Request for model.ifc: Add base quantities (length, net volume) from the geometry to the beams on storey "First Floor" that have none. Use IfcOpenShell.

First a look at what the model holds.

```python
import ifcopenshell
import ifcopenshell.util.element
import ifcopenshell.util.unit

model = ifcopenshell.open("model.ifc")
print(model.schema)
for unit_type in ("LENGTHUNIT", "AREAUNIT", "VOLUMEUNIT"):
    print(unit_type, ifcopenshell.util.unit.calculate_unit_scale(model, unit_type))
storey = next(s for s in model.by_type("IfcBuildingStorey") if s.Name == "First Floor")
beams = [e for e in ifcopenshell.util.element.get_decomposition(storey) if e.is_a("IfcBeam")]
for e in sorted(beams, key=lambda e: e.id()):
    print(e.id(), e.is_a(), e.Name, list(ifcopenshell.util.element.get_psets(e, qtos_only=True)), sep=" | ")
```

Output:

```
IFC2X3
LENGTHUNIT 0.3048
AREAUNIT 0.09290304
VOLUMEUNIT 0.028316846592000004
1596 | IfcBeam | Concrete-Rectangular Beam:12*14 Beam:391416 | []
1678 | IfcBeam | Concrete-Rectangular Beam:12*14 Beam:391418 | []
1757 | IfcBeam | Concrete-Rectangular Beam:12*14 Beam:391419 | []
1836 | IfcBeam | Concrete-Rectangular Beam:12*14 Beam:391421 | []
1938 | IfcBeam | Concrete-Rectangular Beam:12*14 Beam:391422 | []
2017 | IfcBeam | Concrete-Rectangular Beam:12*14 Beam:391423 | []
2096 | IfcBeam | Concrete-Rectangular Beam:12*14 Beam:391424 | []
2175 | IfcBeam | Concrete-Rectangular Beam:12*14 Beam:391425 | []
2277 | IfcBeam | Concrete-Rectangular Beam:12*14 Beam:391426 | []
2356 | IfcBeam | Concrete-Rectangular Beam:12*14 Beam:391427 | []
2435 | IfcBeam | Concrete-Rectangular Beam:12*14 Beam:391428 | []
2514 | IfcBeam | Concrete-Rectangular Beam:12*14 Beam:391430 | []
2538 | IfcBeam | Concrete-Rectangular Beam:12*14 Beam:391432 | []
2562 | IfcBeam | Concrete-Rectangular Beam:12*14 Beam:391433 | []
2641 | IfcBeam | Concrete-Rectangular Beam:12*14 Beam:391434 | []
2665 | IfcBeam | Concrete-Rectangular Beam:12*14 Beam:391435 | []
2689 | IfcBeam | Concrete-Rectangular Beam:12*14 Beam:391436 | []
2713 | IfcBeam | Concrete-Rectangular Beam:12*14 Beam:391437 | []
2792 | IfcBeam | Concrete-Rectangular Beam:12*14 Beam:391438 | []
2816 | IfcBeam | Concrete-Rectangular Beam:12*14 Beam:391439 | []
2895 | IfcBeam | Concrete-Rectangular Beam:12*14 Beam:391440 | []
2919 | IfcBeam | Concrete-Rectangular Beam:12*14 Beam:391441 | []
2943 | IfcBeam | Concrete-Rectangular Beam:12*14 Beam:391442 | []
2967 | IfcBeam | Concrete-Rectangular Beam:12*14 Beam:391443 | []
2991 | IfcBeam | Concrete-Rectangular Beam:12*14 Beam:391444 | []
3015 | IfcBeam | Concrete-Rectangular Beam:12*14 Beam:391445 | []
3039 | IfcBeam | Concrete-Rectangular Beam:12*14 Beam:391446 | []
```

```python
import ifcopenshell
import ifcopenshell.api.pset
import ifcopenshell.geom
import ifcopenshell.util.element
import ifcopenshell.util.shape
import ifcopenshell.util.unit

model = ifcopenshell.open("model.ifc")
unit_scale = ifcopenshell.util.unit.calculate_unit_scale(model)
volume_scale = ifcopenshell.util.unit.calculate_unit_scale(model, "VOLUMEUNIT")
settings = ifcopenshell.geom.settings()

storey = next(s for s in model.by_type("IfcBuildingStorey") if s.Name == "First Floor")
beams = [e for e in ifcopenshell.util.element.get_decomposition(storey) if e.is_a("IfcBeam")]

for e in sorted(beams, key=lambda e: e.id()):
    if ifcopenshell.util.element.get_psets(e, qtos_only=True, should_inherit=False):
        continue
    # Geometry comes back in metres, in the element's own axes.
    shape = ifcopenshell.geom.create_shape(settings, e)
    values = {
        "Length": ifcopenshell.util.shape.get_max_xyz(shape.geometry) / unit_scale,
        "NetVolume": ifcopenshell.util.shape.get_volume(shape.geometry) / volume_scale,
    }
    qto = ifcopenshell.api.pset.add_qto(model, product=e, name="BaseQuantities")
    ifcopenshell.api.pset.edit_qto(model, qto=qto, properties=values)
    print(e.id(), {k: round(v, 3) for k, v in values.items()})

model.write("model_updated.ifc")
```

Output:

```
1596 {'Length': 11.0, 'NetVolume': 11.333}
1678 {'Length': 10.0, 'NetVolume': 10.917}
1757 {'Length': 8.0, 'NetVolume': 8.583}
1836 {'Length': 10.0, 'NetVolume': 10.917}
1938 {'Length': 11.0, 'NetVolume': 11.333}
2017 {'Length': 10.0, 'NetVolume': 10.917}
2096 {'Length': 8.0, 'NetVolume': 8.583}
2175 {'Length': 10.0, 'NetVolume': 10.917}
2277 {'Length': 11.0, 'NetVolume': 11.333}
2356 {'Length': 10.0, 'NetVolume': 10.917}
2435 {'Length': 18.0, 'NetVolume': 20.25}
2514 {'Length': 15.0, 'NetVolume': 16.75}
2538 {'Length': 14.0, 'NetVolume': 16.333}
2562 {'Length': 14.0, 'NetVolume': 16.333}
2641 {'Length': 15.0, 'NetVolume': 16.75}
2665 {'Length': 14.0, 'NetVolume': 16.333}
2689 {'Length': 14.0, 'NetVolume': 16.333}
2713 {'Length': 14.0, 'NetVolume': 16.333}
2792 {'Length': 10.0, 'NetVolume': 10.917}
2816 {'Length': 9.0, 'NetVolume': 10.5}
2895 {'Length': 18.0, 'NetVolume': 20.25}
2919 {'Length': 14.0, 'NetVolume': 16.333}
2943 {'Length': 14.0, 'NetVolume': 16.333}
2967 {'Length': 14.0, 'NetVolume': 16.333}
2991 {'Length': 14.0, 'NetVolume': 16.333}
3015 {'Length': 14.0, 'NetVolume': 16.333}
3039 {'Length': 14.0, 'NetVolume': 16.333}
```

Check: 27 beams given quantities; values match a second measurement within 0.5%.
